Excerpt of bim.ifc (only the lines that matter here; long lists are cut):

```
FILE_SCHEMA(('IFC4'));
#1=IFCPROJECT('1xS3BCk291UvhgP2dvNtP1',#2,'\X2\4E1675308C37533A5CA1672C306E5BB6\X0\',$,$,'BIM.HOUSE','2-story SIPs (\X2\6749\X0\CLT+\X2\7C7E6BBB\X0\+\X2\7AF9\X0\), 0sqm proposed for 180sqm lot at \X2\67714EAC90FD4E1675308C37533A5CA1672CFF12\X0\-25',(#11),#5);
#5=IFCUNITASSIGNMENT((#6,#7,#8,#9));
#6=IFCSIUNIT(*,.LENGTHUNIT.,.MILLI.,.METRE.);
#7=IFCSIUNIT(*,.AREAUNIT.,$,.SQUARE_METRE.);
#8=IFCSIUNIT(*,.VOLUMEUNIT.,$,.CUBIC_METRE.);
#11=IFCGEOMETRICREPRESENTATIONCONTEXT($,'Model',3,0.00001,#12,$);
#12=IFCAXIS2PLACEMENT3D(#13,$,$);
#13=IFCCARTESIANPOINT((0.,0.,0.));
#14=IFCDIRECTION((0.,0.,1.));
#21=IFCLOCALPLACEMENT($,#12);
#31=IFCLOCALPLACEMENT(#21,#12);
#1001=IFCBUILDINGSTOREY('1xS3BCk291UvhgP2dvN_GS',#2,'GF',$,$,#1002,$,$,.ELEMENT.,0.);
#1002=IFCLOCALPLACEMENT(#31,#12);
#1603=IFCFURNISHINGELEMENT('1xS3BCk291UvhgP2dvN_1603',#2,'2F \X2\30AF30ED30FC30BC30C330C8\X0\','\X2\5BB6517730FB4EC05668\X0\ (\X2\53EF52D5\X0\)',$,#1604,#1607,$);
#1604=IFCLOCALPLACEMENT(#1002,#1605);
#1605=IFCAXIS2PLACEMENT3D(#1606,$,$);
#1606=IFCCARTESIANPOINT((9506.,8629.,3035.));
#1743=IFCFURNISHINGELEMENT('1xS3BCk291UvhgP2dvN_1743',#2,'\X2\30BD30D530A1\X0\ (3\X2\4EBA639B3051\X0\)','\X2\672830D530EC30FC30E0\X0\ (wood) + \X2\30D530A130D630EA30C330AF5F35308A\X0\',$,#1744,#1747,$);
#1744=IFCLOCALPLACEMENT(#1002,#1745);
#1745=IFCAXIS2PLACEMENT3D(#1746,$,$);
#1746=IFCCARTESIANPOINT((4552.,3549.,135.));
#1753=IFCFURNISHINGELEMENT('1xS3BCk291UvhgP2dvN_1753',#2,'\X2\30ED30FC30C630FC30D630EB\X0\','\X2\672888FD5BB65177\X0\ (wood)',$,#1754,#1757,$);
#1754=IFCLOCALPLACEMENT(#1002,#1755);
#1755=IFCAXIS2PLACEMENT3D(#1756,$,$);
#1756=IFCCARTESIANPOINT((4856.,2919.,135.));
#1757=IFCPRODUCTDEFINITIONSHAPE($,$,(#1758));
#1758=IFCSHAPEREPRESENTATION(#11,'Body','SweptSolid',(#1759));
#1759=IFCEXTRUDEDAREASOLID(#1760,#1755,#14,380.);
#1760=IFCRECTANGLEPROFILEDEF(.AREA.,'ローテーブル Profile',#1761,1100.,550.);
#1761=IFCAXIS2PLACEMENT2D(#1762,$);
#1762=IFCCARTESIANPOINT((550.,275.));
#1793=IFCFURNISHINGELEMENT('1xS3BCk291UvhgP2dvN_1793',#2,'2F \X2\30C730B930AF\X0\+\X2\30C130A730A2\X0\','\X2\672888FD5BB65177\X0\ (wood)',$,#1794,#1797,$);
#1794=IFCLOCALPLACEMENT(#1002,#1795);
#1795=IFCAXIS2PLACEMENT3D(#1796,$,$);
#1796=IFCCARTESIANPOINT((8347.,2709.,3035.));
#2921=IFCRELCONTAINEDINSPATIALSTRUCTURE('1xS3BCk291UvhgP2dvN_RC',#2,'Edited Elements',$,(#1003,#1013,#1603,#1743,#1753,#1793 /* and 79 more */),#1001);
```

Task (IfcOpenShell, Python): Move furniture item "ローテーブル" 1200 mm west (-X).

```python
import ifcopenshell
import ifcopenshell.api.geometry
import ifcopenshell.util.placement
import ifcopenshell.util.unit

model = ifcopenshell.open("bim.ifc")
unit_scale = ifcopenshell.util.unit.calculate_unit_scale(model)

item = model.by_guid("1xS3BCk291UvhgP2dvN_1753")
matrix = ifcopenshell.util.placement.get_local_placement(item.ObjectPlacement)
matrix[0, 3] -= 1.2 / unit_scale
ifcopenshell.api.geometry.edit_object_placement(model, product=item, matrix=matrix, is_si=False)

print(ifcopenshell.util.placement.get_local_placement(item.ObjectPlacement).round(3) + 0.0)

model.write("bim_updated.ifc")
```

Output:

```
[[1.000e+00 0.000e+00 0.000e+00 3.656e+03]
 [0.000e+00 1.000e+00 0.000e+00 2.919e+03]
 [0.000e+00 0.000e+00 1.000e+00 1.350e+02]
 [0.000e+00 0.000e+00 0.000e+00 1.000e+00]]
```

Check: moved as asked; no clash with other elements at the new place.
